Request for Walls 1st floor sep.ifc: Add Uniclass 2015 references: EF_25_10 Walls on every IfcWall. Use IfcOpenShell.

First a look at what the model holds.

```python
import ifcopenshell

model = ifcopenshell.open("Walls 1st floor sep.ifc")
print(model.schema)
print("classifications:", [c.Name for c in model.by_type("IfcClassification")])
for ifc_class in ("IfcDoor", "IfcRoof", "IfcStair", "IfcWall", "IfcWindow"):
    print(ifc_class, len(model.by_type(ifc_class)))
```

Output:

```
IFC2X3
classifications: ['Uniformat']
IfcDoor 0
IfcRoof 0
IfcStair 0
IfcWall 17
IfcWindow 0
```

```python
import ifcopenshell
import ifcopenshell.api.classification

model = ifcopenshell.open("Walls 1st floor sep.ifc")

# IFC2X3 requires Source and Edition and has no link from the project to the system.
system = model.create_entity("IfcClassification", Source="NBS", Edition="2015", Name="Uniclass 2015")

codes = {
    "IfcWall": ("EF_25_10", "Walls"),
}
for ifc_class, (code, name) in codes.items():
    products = model.by_type(ifc_class)
    ifcopenshell.api.classification.add_reference(
        model, products=products, classification=system, identification=code, name=name
    )
    print(code, len(products))

model.write("Walls 1st floor sep_edited.ifc")
```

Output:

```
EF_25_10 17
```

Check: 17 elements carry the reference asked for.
